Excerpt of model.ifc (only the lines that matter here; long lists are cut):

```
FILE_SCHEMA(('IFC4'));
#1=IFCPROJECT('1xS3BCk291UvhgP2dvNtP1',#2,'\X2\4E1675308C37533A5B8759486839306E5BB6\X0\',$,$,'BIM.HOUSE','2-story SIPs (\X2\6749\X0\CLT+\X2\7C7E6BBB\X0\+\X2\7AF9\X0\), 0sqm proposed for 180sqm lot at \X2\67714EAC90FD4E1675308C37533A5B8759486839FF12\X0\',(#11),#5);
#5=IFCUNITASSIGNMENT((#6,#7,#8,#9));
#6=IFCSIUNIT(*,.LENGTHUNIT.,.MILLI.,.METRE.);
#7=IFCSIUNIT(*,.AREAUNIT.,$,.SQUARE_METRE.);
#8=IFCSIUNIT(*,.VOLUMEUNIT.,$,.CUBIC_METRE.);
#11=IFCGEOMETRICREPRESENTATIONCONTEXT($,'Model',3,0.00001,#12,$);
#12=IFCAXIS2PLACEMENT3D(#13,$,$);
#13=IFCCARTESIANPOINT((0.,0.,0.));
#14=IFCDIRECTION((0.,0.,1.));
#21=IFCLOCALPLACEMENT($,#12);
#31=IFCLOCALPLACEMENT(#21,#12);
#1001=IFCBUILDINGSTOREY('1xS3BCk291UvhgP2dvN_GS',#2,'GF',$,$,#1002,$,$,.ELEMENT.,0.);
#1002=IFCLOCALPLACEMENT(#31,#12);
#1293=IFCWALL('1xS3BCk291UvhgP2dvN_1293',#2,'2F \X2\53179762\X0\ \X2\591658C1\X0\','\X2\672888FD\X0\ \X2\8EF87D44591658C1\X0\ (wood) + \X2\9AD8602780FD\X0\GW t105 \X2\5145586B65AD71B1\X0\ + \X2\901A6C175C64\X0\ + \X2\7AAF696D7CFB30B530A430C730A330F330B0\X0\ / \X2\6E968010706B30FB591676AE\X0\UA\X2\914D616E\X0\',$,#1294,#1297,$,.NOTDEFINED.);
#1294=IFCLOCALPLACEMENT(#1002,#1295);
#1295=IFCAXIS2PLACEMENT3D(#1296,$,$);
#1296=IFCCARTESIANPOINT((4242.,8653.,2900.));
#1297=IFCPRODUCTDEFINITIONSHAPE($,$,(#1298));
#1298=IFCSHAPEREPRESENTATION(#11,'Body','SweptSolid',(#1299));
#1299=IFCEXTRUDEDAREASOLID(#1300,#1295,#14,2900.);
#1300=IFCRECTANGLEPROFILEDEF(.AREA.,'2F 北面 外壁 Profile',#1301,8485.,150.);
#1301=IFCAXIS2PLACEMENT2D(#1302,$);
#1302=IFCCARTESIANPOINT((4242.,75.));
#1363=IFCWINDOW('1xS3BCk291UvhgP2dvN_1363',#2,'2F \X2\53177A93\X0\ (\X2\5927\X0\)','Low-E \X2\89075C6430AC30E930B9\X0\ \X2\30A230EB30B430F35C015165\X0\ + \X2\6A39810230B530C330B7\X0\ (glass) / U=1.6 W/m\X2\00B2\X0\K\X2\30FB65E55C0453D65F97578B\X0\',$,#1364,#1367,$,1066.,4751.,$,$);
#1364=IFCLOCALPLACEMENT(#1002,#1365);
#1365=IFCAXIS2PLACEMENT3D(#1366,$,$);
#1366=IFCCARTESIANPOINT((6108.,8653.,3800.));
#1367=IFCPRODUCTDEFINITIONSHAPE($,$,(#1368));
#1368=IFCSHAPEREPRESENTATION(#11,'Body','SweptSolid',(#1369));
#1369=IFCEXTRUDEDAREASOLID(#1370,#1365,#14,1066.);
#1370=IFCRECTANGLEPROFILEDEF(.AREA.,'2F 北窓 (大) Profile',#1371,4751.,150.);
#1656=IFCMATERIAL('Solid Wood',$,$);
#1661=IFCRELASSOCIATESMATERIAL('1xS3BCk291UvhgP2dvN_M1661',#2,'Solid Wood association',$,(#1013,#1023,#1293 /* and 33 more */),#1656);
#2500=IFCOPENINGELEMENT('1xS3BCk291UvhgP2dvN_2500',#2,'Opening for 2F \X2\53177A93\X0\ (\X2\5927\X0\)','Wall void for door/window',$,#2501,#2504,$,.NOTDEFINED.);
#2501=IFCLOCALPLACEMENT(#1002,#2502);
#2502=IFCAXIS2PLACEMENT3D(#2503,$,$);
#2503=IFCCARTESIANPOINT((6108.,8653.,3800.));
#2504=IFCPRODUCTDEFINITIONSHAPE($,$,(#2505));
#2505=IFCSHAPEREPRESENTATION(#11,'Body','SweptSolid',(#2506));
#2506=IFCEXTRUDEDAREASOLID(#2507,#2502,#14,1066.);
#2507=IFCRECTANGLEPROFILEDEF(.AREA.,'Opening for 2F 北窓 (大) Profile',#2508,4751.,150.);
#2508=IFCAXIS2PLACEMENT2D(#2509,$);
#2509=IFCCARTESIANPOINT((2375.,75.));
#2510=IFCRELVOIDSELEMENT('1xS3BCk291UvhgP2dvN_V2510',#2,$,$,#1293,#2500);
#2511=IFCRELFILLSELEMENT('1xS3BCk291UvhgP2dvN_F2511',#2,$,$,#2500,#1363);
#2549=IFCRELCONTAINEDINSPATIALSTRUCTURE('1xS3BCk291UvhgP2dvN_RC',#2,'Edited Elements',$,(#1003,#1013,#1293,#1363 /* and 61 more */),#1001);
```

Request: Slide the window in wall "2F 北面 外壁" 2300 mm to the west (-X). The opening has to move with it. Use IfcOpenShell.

```python
import ifcopenshell
import ifcopenshell.api.geometry
import ifcopenshell.util.placement
import ifcopenshell.util.unit

model = ifcopenshell.open("model.ifc")
unit_scale = ifcopenshell.util.unit.calculate_unit_scale(model)

window = model.by_guid("1xS3BCk291UvhgP2dvN_1363")
opening = window.FillsVoids[0].RelatingOpeningElement
wall = opening.VoidsElements[0].RelatingBuildingElement

wall_matrix = ifcopenshell.util.placement.get_local_placement(wall.ObjectPlacement)
shift = wall_matrix[:3, 0] * -2.3 / unit_scale
before = ifcopenshell.util.placement.get_local_placement(window.ObjectPlacement)[:3, 3].copy()

# The window is not placed relative to its opening, so move both.
for product in (opening, window):
    matrix = ifcopenshell.util.placement.get_local_placement(product.ObjectPlacement)
    matrix[:3, 3] += shift
    ifcopenshell.api.geometry.edit_object_placement(model, product=product, matrix=matrix, is_si=False)

after = ifcopenshell.util.placement.get_local_placement(window.ObjectPlacement)[:3, 3]
print("window moved by", (after - before).round(3) + 0.0)

model.write("model_v2.ifc")
```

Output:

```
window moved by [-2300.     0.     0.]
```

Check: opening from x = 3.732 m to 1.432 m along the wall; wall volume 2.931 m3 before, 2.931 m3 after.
